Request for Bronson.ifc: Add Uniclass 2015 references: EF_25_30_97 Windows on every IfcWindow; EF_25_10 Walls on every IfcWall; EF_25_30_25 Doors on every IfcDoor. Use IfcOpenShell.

First a look at what the model holds.

```python
import ifcopenshell

model = ifcopenshell.open("Bronson.ifc")
print(model.schema)
print("classifications:", [c.Name for c in model.by_type("IfcClassification")])
for ifc_class in ("IfcDoor", "IfcRoof", "IfcStair", "IfcWall", "IfcWindow"):
    print(ifc_class, len(model.by_type(ifc_class)))
```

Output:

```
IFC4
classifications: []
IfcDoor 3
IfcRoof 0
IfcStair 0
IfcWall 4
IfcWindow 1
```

```python
import ifcopenshell
import ifcopenshell.api.classification

model = ifcopenshell.open("Bronson.ifc")

system = ifcopenshell.api.classification.add_classification(model, classification="Uniclass 2015")

codes = {
    "IfcWindow": ("EF_25_30_97", "Windows"),
    "IfcWall": ("EF_25_10", "Walls"),
    "IfcDoor": ("EF_25_30_25", "Doors"),
}
for ifc_class, (code, name) in codes.items():
    products = model.by_type(ifc_class)
    ifcopenshell.api.classification.add_reference(
        model, products=products, classification=system, identification=code, name=name
    )
    print(code, len(products))

model.write("Bronson_v2.ifc")
```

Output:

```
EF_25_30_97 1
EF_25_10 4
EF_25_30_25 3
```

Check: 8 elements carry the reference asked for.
